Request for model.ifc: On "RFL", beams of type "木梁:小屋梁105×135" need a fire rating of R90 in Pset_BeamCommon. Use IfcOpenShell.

First a look at what the model holds.

```python
import ifcopenshell
import ifcopenshell.util.element

model = ifcopenshell.open("model.ifc")
print(model.schema)
storey = next(s for s in model.by_type("IfcBuildingStorey") if s.Name == "RFL")
beams = [e for e in ifcopenshell.util.element.get_decomposition(storey) if e.is_a("IfcBeam")]
seen = {}
for e in beams:
    element_type = ifcopenshell.util.element.get_type(e)
    key = (element_type.Name if element_type != e and element_type else None, ifcopenshell.util.element.get_pset(e, "Pset_BeamCommon", "FireRating"))
    seen[key] = seen.get(key, 0) + 1
for (name, value), count in sorted(seen.items(), key=str):
    print(count, "x", name, "|", value)
```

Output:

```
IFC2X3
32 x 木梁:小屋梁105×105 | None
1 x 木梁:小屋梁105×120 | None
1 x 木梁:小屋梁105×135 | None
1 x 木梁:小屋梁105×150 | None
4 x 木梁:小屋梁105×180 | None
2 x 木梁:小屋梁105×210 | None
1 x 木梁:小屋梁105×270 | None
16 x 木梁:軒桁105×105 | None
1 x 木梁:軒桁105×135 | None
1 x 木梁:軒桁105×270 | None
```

```python
import ifcopenshell
import ifcopenshell.api.pset
import ifcopenshell.util.element

model = ifcopenshell.open("model.ifc")

storey = next(s for s in model.by_type("IfcBuildingStorey") if s.Name == "RFL")
beams = [e for e in ifcopenshell.util.element.get_decomposition(storey) if e.is_a("IfcBeam")]

count = 0
for e in beams:
    element_type = ifcopenshell.util.element.get_type(e)
    if element_type in (None, e) or element_type.Name != "木梁:小屋梁105×135":
        continue
    # add_pset returns the element's existing set when there is one.
    pset = ifcopenshell.api.pset.add_pset(model, product=e, name="Pset_BeamCommon")
    ifcopenshell.api.pset.edit_pset(model, pset=pset, properties={"FireRating": "R90"})
    count += 1

print(count, "beams updated")

model.write("model_edited.ifc")
```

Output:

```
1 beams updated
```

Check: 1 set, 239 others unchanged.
